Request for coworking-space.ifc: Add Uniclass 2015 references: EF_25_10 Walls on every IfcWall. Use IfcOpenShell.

First a look at what the model holds.

```python
import ifcopenshell

model = ifcopenshell.open("coworking-space.ifc")
print(model.schema)
print("classifications:", [c.Name for c in model.by_type("IfcClassification")])
for ifc_class in ("IfcDoor", "IfcRoof", "IfcStair", "IfcWall", "IfcWindow"):
    print(ifc_class, len(model.by_type(ifc_class)))
```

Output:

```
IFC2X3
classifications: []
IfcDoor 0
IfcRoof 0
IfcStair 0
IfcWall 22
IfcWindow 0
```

```python
import ifcopenshell
import ifcopenshell.api.classification

model = ifcopenshell.open("coworking-space.ifc")

# IFC2X3 requires Source and Edition and has no link from the project to the system.
system = model.create_entity("IfcClassification", Source="NBS", Edition="2015", Name="Uniclass 2015")

codes = {
    "IfcWall": ("EF_25_10", "Walls"),
}
for ifc_class, (code, name) in codes.items():
    products = model.by_type(ifc_class)
    ifcopenshell.api.classification.add_reference(
        model, products=products, classification=system, identification=code, name=name
    )
    print(code, len(products))

model.write("coworking-space_v2.ifc")
```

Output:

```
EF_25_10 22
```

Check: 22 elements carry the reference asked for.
